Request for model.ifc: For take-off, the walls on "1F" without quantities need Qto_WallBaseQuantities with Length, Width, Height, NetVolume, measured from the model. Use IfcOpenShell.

First a look at what the model holds.

```python
import ifcopenshell
import ifcopenshell.util.element
import ifcopenshell.util.unit

model = ifcopenshell.open("model.ifc")
print(model.schema)
for unit_type in ("LENGTHUNIT", "AREAUNIT", "VOLUMEUNIT"):
    print(unit_type, ifcopenshell.util.unit.calculate_unit_scale(model, unit_type))
storey = next(s for s in model.by_type("IfcBuildingStorey") if s.Name == "1F")
walls = [e for e in ifcopenshell.util.element.get_decomposition(storey) if e.is_a("IfcWall")]
for e in sorted(walls, key=lambda e: e.id()):
    print(e.id(), e.is_a(), e.Name, list(ifcopenshell.util.element.get_psets(e, qtos_only=True)), sep=" | ")
```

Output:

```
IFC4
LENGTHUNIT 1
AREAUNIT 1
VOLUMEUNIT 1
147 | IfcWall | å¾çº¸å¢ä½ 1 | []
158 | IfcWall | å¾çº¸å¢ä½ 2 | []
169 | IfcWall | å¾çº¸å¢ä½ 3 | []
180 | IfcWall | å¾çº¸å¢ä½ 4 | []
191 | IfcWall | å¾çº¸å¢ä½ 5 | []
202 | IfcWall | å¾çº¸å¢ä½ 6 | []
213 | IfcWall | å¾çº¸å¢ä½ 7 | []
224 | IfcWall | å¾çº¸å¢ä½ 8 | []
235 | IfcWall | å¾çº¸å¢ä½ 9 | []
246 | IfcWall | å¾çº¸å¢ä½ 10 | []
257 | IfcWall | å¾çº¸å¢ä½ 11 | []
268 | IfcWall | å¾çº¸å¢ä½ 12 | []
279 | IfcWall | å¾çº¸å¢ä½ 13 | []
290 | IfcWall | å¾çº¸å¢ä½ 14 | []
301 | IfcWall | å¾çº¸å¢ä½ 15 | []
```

```python
import ifcopenshell
import ifcopenshell.api.pset
import ifcopenshell.geom
import ifcopenshell.util.element
import ifcopenshell.util.shape
import ifcopenshell.util.unit

model = ifcopenshell.open("model.ifc")
unit_scale = ifcopenshell.util.unit.calculate_unit_scale(model)
volume_scale = ifcopenshell.util.unit.calculate_unit_scale(model, "VOLUMEUNIT")
settings = ifcopenshell.geom.settings()

storey = next(s for s in model.by_type("IfcBuildingStorey") if s.Name == "1F")
walls = [e for e in ifcopenshell.util.element.get_decomposition(storey) if e.is_a("IfcWall")]

for e in sorted(walls, key=lambda e: e.id()):
    if ifcopenshell.util.element.get_psets(e, qtos_only=True, should_inherit=False):
        continue
    # Geometry comes back in metres, in the element's own axes.
    shape = ifcopenshell.geom.create_shape(settings, e)
    values = {
        "Length": ifcopenshell.util.shape.get_x(shape.geometry) / unit_scale,
        "Width": ifcopenshell.util.shape.get_y(shape.geometry) / unit_scale,
        "Height": ifcopenshell.util.shape.get_z(shape.geometry) / unit_scale,
        "NetVolume": ifcopenshell.util.shape.get_volume(shape.geometry) / volume_scale,
    }
    qto = ifcopenshell.api.pset.add_qto(model, product=e, name="Qto_WallBaseQuantities")
    ifcopenshell.api.pset.edit_qto(model, qto=qto, properties=values)
    print(e.id(), {k: round(v, 3) for k, v in values.items()})

model.write("model_v2.ifc")
```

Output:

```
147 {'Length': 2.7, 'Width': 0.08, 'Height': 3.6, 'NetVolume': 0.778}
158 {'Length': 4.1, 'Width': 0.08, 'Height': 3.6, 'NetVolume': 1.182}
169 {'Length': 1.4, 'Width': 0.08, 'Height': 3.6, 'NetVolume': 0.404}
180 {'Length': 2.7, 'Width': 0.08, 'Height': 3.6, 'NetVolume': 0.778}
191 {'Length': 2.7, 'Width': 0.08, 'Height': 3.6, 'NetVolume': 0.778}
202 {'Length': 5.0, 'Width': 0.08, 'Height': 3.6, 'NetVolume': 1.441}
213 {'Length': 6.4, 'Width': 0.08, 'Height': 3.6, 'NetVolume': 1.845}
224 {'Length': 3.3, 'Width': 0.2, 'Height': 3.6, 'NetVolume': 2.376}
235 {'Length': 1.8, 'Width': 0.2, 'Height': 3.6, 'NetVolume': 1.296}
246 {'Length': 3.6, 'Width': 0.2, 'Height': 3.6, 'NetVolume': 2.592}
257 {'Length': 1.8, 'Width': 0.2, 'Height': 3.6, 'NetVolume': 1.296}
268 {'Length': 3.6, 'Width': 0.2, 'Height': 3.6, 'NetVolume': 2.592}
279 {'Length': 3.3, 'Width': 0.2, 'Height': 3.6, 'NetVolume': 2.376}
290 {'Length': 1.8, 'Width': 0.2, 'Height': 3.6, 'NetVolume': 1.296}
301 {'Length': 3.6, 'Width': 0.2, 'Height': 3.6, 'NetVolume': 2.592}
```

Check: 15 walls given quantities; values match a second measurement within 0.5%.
